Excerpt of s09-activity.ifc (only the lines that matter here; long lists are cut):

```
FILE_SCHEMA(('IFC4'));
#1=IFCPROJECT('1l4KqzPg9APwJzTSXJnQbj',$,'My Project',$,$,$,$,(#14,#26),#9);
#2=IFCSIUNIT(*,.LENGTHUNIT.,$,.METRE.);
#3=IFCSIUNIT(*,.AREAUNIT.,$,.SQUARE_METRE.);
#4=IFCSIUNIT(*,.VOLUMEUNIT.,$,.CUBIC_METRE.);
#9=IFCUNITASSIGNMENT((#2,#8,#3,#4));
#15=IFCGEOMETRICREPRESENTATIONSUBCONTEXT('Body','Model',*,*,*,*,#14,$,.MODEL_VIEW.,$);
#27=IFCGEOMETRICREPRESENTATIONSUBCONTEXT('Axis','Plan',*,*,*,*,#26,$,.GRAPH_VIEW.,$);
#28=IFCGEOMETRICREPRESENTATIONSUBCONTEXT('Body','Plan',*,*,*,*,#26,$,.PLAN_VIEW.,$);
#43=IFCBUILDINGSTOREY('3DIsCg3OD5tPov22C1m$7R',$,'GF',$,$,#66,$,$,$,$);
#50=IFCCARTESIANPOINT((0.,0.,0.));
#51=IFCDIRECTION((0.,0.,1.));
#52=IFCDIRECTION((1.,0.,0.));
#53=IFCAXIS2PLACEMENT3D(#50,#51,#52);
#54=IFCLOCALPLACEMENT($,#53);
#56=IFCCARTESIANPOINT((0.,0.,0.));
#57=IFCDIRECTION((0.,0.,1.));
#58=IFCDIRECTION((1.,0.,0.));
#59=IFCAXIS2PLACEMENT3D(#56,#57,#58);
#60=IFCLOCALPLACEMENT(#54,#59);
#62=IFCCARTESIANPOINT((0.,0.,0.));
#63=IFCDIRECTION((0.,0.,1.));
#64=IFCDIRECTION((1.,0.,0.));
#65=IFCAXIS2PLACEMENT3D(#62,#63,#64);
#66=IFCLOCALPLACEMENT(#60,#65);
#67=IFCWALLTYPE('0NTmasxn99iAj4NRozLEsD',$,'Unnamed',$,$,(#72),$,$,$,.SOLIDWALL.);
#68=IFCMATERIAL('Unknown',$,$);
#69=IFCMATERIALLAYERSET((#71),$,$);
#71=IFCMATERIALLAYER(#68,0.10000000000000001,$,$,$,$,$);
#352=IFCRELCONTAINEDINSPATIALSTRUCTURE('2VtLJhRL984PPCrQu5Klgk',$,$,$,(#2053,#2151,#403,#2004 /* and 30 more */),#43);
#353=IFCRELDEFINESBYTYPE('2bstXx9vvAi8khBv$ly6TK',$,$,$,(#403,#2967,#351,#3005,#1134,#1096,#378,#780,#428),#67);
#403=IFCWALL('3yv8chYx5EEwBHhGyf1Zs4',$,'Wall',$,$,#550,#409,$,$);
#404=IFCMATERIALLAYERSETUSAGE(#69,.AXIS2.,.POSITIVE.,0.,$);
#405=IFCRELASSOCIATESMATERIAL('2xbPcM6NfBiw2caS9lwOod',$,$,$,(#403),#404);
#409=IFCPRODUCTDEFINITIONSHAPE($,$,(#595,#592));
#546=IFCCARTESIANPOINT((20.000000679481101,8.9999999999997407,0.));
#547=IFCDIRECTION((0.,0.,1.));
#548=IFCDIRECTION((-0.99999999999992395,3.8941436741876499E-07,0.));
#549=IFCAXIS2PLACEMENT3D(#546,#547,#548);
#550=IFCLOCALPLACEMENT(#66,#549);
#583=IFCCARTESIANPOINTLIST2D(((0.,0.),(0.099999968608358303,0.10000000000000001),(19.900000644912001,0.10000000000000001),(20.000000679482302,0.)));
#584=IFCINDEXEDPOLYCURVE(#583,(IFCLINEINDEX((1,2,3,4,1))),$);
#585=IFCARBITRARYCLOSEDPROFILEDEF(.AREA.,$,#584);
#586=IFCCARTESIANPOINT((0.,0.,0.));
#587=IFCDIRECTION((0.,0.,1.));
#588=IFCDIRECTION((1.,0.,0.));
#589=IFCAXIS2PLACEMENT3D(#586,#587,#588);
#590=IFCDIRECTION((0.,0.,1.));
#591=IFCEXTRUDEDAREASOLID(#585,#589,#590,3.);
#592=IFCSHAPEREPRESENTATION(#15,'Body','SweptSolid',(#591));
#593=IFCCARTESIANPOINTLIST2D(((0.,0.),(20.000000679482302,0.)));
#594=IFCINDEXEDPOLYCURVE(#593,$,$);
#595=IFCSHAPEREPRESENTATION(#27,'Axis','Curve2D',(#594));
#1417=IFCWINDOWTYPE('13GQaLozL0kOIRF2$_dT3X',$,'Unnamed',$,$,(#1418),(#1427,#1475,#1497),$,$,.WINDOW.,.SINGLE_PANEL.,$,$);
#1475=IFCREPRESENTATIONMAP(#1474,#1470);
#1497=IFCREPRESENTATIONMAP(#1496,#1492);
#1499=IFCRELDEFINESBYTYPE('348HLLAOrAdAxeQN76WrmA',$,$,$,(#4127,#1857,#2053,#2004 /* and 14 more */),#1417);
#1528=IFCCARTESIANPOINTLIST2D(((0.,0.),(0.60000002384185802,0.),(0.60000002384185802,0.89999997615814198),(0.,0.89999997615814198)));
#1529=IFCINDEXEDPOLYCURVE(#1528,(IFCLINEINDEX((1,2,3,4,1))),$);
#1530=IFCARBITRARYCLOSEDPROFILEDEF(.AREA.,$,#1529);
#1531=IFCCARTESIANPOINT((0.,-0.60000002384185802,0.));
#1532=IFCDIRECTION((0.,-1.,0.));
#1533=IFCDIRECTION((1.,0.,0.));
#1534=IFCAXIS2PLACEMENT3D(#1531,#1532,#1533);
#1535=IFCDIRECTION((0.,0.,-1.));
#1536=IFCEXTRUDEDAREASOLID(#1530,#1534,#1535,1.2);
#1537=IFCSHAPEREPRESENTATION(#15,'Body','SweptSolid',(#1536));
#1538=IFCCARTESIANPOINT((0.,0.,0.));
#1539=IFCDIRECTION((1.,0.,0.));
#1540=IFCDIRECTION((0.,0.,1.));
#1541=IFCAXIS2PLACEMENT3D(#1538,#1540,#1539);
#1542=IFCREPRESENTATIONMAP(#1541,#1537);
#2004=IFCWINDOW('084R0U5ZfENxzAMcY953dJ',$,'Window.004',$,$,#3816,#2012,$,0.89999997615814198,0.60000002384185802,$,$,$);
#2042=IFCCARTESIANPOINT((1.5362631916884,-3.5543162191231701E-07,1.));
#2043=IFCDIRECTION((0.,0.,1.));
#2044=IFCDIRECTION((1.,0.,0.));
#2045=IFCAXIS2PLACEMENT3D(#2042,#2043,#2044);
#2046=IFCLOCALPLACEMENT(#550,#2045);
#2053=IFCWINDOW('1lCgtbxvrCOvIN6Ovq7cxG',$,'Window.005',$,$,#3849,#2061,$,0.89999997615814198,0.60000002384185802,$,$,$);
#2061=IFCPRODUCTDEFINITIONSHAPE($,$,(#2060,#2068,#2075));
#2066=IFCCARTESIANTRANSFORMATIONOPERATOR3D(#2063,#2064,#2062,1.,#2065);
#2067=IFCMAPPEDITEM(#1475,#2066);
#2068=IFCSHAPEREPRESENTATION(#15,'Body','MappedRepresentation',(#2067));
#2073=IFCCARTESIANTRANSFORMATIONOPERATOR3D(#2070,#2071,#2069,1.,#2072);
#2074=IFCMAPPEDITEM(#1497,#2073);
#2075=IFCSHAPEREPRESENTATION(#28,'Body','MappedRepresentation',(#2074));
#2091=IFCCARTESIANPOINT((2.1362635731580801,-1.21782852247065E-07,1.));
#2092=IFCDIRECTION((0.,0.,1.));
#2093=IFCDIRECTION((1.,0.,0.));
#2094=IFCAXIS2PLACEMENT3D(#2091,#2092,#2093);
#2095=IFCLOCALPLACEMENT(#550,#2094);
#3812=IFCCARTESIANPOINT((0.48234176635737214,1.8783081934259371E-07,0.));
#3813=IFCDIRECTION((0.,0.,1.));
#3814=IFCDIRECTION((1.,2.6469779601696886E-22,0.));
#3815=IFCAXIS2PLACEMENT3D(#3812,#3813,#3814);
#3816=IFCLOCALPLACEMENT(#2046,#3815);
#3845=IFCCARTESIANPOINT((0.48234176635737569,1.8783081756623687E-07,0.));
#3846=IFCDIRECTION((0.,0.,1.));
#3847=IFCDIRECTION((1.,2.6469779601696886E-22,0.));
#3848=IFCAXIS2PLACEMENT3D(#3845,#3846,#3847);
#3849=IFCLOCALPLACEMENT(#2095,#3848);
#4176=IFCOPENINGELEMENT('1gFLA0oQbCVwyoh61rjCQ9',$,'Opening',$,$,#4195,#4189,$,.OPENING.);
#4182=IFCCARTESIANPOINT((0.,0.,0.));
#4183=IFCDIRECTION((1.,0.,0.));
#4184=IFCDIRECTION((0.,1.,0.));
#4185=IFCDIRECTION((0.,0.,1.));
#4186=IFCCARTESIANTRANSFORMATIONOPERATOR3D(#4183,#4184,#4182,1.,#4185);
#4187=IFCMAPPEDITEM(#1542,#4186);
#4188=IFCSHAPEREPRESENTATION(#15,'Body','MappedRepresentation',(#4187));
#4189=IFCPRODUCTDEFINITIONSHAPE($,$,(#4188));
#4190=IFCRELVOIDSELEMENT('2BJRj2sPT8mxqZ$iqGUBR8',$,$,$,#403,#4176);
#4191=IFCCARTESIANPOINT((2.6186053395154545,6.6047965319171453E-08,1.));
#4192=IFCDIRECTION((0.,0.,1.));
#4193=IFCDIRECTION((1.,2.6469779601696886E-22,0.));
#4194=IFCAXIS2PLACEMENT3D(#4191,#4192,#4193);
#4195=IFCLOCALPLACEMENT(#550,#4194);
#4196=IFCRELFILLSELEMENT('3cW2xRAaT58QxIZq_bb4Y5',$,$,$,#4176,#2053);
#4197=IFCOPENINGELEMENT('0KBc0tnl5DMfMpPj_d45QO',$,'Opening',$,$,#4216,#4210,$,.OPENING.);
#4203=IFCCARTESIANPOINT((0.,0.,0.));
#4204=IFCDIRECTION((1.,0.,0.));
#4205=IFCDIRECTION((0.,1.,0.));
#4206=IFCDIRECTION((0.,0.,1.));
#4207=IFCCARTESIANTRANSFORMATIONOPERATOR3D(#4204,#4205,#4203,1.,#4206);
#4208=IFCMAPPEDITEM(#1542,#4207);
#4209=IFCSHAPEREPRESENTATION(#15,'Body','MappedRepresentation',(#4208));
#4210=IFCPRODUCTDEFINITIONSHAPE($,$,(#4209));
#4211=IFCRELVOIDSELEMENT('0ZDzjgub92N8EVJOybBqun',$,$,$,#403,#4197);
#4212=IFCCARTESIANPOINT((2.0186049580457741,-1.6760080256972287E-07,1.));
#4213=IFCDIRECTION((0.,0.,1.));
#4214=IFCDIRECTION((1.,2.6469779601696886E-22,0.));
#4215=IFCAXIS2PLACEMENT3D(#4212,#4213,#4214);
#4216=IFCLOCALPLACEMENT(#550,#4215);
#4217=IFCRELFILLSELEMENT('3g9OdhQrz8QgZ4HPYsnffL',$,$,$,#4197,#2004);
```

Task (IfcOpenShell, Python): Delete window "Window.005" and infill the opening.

```python
import ifcopenshell
import ifcopenshell.api.feature
import ifcopenshell.api.root
import ifcopenshell.geom
import ifcopenshell.util.shape

model = ifcopenshell.open("s09-activity.ifc")
settings = ifcopenshell.geom.settings()


def volume(element):
    """Net volume in cubic metres, openings subtracted."""
    shape = ifcopenshell.geom.create_shape(settings, element)
    return ifcopenshell.util.shape.get_volume(shape.geometry)


window = model.by_guid("1lCgtbxvrCOvIN6Ovq7cxG")
opening = window.FillsVoids[0].RelatingOpeningElement
wall = opening.VoidsElements[0].RelatingBuildingElement
before = volume(wall)

ifcopenshell.api.root.remove_product(model, product=window)
ifcopenshell.api.feature.remove_feature(model, feature=opening)

after = volume(wall)

print(f"wall volume {before:.3f} -> {after:.3f} m3")

model.write("s09-activity_updated.ifc")
```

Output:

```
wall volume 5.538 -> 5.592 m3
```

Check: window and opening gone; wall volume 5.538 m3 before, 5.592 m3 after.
